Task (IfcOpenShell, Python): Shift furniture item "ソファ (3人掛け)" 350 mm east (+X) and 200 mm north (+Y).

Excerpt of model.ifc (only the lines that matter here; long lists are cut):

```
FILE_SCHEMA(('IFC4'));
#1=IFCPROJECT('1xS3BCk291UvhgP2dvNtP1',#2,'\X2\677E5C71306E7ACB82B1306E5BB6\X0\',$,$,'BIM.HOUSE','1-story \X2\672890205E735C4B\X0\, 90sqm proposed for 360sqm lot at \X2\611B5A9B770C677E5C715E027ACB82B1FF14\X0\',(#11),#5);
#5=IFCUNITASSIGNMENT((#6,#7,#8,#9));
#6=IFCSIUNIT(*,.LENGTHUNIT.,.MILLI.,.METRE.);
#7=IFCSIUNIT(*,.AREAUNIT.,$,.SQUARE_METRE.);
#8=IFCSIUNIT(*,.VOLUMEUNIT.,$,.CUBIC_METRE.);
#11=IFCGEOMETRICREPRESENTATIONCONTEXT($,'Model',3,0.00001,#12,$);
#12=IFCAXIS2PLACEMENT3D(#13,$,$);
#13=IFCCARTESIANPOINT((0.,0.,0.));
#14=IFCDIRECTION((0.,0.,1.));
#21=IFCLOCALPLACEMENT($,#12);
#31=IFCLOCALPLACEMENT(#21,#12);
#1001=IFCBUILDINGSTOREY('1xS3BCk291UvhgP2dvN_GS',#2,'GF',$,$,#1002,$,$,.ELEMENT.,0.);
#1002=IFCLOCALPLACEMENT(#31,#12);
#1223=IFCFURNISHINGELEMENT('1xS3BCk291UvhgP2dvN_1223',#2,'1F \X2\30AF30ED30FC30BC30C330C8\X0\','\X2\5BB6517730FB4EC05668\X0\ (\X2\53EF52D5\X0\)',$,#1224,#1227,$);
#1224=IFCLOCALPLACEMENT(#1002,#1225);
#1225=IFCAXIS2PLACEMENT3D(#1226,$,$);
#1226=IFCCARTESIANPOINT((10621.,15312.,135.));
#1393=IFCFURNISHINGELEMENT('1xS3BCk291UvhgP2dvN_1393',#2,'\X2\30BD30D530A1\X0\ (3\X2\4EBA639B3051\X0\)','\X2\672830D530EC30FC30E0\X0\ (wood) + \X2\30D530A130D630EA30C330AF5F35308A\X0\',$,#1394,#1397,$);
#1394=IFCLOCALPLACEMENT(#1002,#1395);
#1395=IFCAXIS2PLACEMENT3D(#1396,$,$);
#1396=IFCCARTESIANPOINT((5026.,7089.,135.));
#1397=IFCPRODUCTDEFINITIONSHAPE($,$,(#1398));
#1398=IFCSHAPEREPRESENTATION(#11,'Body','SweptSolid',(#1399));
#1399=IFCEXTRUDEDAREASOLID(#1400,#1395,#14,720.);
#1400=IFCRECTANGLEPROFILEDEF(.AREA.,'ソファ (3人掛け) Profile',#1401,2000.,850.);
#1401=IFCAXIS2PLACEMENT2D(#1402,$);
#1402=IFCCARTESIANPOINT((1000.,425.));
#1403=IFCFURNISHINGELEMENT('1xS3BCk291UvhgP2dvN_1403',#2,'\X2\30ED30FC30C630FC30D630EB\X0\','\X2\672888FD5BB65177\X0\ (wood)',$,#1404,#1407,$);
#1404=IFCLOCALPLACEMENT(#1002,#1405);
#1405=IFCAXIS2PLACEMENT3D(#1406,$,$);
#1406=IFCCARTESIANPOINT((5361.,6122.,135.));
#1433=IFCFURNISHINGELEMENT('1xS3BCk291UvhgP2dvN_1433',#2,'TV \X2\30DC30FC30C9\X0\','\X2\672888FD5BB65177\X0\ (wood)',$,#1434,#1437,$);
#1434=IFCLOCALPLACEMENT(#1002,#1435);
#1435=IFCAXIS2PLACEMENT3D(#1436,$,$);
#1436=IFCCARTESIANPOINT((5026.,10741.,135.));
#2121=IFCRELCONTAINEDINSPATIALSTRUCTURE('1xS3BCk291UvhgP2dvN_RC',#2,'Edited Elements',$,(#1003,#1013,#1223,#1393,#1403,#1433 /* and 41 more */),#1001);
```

```python
import ifcopenshell
import ifcopenshell.api.geometry
import ifcopenshell.util.placement

model = ifcopenshell.open("model.ifc")

item = model.by_guid("1xS3BCk291UvhgP2dvN_1393")
matrix = ifcopenshell.util.placement.get_local_placement(item.ObjectPlacement)
matrix[0, 3] += 350.0
matrix[1, 3] += 200.0
ifcopenshell.api.geometry.edit_object_placement(model, product=item, matrix=matrix, is_si=False)

print(ifcopenshell.util.placement.get_local_placement(item.ObjectPlacement).round(3) + 0.0)

model.write("model_updated.ifc")
```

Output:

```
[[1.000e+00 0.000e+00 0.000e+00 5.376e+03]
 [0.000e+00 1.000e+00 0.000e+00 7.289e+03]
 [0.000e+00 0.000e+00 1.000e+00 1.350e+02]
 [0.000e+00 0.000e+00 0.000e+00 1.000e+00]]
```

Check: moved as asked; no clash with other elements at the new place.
